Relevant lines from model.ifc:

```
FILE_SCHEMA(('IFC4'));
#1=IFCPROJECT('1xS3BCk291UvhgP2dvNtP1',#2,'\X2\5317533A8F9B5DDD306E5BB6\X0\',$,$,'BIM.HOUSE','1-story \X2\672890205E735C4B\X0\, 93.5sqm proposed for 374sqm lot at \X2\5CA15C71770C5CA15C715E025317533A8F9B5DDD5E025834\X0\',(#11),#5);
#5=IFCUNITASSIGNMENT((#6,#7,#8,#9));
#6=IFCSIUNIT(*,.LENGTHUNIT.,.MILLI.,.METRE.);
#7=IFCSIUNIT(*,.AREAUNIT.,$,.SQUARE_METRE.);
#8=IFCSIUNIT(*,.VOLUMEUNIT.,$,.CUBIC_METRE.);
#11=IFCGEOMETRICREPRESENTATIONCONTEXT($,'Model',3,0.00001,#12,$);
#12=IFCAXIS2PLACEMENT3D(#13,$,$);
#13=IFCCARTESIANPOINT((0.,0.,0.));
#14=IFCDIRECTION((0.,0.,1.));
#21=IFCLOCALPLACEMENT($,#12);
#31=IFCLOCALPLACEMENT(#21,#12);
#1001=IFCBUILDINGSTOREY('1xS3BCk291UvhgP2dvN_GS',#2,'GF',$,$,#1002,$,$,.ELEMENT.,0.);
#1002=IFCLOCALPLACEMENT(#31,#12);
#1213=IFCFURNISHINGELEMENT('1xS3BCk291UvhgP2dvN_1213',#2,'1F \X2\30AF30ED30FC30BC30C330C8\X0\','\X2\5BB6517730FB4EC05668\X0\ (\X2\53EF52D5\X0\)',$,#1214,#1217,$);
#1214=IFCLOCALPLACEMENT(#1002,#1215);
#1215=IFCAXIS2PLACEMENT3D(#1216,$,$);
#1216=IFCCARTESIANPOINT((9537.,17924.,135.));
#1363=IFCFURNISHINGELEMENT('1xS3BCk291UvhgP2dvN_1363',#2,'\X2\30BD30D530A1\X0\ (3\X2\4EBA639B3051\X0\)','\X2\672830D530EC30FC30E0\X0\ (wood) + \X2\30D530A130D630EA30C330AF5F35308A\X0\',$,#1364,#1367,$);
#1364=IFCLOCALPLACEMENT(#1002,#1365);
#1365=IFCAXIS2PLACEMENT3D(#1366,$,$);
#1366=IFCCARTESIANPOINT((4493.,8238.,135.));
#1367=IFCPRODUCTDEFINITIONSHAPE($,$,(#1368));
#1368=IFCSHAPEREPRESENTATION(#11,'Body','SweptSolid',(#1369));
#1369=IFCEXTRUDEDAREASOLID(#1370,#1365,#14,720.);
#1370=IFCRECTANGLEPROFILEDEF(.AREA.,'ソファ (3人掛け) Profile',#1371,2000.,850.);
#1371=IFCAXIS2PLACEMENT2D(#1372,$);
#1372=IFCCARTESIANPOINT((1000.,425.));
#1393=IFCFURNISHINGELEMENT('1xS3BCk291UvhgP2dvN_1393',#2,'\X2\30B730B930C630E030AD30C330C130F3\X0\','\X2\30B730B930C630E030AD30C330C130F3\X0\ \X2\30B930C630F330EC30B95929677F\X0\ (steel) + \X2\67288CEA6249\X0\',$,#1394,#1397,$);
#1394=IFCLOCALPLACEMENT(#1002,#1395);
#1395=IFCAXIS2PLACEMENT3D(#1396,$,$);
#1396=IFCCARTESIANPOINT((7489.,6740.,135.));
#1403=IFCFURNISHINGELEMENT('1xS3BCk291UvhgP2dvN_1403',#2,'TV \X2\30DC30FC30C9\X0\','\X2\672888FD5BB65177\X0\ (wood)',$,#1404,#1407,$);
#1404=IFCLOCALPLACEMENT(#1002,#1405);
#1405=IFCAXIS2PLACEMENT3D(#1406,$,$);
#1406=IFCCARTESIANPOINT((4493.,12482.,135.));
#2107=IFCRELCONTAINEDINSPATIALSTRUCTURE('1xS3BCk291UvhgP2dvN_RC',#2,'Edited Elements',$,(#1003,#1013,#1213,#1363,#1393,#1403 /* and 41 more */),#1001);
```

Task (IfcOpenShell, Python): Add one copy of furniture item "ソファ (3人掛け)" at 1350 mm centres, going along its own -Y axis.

```python
import ifcopenshell
import ifcopenshell.api.geometry
import ifcopenshell.api.root
import ifcopenshell.util.element
import ifcopenshell.util.placement
import ifcopenshell.util.unit

model = ifcopenshell.open("model.ifc")
unit_scale = ifcopenshell.util.unit.calculate_unit_scale(model)


def reuse_history(source, copy):
    """copy_class also copies each property set's owner history, people and application; keep the originals."""
    for rel in copy.IsDefinedBy:
        if rel.is_a("IfcRelDefinesByProperties") and (history := rel.RelatingPropertyDefinition.OwnerHistory):
            rel.RelatingPropertyDefinition.OwnerHistory = source.OwnerHistory
            ifcopenshell.util.element.remove_deep2(model, history)


source = model.by_id(1363)
base = ifcopenshell.util.placement.get_local_placement(source.ObjectPlacement)
step = -base[:3, 1] * 1.35 / unit_scale

for i in range(1, 2):
    copy = ifcopenshell.api.root.copy_class(model, product=source)
    copy.Representation = ifcopenshell.util.element.copy_deep(
        model, source.Representation, exclude=["IfcGeometricRepresentationContext", "IfcRepresentationMap"]
    )
    reuse_history(source, copy)
    matrix = base.copy()
    matrix[:3, 3] += i * step
    print("added at", matrix[:3, 3].round(3) + 0.0)
    ifcopenshell.api.geometry.edit_object_placement(model, product=copy, matrix=matrix, is_si=False)

model.write("model-out.ifc")
```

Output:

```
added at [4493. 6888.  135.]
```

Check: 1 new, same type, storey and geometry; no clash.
